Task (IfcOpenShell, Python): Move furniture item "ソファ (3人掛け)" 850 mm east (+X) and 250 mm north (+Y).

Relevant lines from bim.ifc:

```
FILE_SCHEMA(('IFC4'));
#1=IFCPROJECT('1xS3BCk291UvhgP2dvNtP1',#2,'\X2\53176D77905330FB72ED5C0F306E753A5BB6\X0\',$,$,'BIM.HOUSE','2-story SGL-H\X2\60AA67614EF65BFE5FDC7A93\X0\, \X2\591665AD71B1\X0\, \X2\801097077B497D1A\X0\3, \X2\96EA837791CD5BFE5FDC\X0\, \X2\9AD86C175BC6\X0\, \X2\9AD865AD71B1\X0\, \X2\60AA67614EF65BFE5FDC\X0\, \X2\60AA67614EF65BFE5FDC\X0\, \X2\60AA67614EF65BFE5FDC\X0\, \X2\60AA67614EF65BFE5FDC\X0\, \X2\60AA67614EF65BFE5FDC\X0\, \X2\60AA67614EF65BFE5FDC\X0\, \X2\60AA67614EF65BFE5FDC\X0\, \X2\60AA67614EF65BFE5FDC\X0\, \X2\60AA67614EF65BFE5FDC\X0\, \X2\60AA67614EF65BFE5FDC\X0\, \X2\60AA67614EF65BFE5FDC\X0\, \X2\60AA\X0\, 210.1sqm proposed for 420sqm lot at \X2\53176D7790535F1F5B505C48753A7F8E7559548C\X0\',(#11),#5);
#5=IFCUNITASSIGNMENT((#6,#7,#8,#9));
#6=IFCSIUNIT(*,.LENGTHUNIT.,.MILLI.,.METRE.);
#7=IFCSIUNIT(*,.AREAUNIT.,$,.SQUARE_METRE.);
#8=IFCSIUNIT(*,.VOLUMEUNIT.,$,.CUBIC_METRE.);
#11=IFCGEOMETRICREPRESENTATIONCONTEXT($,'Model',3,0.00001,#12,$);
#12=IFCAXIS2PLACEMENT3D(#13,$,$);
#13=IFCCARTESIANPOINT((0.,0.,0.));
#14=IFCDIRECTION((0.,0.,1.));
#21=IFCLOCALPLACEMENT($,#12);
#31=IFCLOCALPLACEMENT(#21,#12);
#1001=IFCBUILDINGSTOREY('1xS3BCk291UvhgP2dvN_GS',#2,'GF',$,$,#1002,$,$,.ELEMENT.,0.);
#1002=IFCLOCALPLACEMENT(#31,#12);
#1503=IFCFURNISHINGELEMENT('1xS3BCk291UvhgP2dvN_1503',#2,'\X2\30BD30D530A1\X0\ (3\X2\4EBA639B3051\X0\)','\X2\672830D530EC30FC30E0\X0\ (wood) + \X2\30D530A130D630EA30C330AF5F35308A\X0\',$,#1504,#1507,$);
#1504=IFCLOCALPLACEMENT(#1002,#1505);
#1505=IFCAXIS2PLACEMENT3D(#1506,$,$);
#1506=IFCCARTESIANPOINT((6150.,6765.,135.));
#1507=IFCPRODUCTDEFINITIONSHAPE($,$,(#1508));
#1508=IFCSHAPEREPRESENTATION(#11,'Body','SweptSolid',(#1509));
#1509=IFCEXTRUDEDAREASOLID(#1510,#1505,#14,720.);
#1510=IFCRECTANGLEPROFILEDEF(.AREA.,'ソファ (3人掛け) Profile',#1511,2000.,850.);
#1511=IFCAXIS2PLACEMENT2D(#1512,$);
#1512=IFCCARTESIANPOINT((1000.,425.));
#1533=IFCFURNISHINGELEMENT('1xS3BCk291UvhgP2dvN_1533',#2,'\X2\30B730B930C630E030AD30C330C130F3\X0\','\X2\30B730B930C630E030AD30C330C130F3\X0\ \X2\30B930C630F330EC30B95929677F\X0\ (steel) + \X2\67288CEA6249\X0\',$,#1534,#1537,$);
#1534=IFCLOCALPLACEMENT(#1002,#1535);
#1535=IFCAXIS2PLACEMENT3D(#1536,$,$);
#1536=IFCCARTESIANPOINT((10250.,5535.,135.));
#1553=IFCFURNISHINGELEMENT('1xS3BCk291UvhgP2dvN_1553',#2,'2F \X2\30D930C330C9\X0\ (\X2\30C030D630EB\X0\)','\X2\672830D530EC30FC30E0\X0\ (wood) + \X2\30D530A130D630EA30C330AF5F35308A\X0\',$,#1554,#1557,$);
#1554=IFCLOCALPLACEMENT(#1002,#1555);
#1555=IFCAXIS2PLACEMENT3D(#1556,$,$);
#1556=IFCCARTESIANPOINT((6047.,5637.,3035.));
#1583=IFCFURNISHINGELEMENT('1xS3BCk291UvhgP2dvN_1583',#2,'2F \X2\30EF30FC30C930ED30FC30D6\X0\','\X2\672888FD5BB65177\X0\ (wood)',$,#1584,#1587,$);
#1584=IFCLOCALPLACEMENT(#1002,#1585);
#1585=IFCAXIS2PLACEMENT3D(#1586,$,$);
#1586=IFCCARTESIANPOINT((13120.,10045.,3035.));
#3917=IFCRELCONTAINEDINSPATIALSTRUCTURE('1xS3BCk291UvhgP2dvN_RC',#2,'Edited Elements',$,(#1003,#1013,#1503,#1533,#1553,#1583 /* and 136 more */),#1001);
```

```python
import ifcopenshell
import ifcopenshell.api.geometry
import ifcopenshell.util.placement
import ifcopenshell.util.unit

model = ifcopenshell.open("bim.ifc")
unit_scale = ifcopenshell.util.unit.calculate_unit_scale(model)

item = model.by_guid("1xS3BCk291UvhgP2dvN_1503")
matrix = ifcopenshell.util.placement.get_local_placement(item.ObjectPlacement)
matrix[0, 3] += 0.85 / unit_scale
matrix[1, 3] += 0.25 / unit_scale
ifcopenshell.api.geometry.edit_object_placement(model, product=item, matrix=matrix, is_si=False)

print(ifcopenshell.util.placement.get_local_placement(item.ObjectPlacement).round(3) + 0.0)

model.write("bim-out.ifc")
```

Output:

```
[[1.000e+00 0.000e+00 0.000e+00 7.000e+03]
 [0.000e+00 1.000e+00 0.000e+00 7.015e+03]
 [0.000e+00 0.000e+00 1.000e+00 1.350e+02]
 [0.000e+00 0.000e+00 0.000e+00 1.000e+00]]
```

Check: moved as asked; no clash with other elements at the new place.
